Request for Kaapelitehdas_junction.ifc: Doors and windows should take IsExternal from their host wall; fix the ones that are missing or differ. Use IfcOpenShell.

First a look at what the model holds.

```python
import ifcopenshell
import ifcopenshell.util.element

model = ifcopenshell.open("Kaapelitehdas_junction.ifc")
print(model.schema)
seen = {}
for e in model.by_type("IfcDoor") + model.by_type("IfcWindow"):
    if not e.FillsVoids:
        continue
    host = e.FillsVoids[0].RelatingOpeningElement.VoidsElements[0].RelatingBuildingElement
    own = ifcopenshell.util.element.get_pset(e, f"Pset_{e.is_a()[3:].removesuffix('StandardCase')}Common", "IsExternal")
    wall = ifcopenshell.util.element.get_pset(host, "Pset_WallCommon", "IsExternal")
    seen[e.is_a(), own, wall] = seen.get((e.is_a(), own, wall), 0) + 1
for (cls, own, wall), count in sorted(seen.items(), key=str):
    print(count, cls, "IsExternal:", own, "| host wall:", wall)
```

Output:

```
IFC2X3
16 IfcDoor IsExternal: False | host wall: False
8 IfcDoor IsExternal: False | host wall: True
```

```python
import ifcopenshell
import ifcopenshell.api.pset
import ifcopenshell.util.element

model = ifcopenshell.open("Kaapelitehdas_junction.ifc")

count = 0
for ifc_class, pset_name in (("IfcDoor", "Pset_DoorCommon"), ("IfcWindow", "Pset_WindowCommon")):
    for e in model.by_type(ifc_class):
        if not e.FillsVoids:
            continue
        host = e.FillsVoids[0].RelatingOpeningElement.VoidsElements[0].RelatingBuildingElement
        external = ifcopenshell.util.element.get_pset(host, "Pset_WallCommon", "IsExternal")
        if external is None or ifcopenshell.util.element.get_pset(e, pset_name, "IsExternal") == external:
            continue
        pset = ifcopenshell.api.pset.add_pset(model, product=e, name=pset_name)
        ifcopenshell.api.pset.edit_pset(model, pset=pset, properties={"IsExternal": external})
        count += 1

print(count, "updated")

model.write("Kaapelitehdas_junction_v2.ifc")
```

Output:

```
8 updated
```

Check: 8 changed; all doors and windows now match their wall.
